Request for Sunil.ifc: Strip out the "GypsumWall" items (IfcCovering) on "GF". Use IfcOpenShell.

First a look at what the model holds.

```python
import ifcopenshell
import ifcopenshell.util.element

model = ifcopenshell.open("Sunil.ifc")
print(model.schema)
storey = next(s for s in model.by_type("IfcBuildingStorey") if s.Name == "GF")
coverings = [e for e in ifcopenshell.util.element.get_decomposition(storey) if e.is_a("IfcCovering")]
seen = {}
for e in coverings:
    element_type = ifcopenshell.util.element.get_type(e)
    name = element_type.Name if element_type not in (None, e) else None
    seen[name] = seen.get(name, 0) + 1
for name, count in sorted(seen.items(), key=str):
    print(count, "x", name)
```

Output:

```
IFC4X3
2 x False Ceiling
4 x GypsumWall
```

```python
import ifcopenshell
import ifcopenshell.api.root
import ifcopenshell.util.element

model = ifcopenshell.open("Sunil.ifc")

storey = next(s for s in model.by_type("IfcBuildingStorey") if s.Name == "GF")
coverings = [e for e in ifcopenshell.util.element.get_decomposition(storey) if e.is_a("IfcCovering")]
targets = [e for e in coverings if (t := ifcopenshell.util.element.get_type(e)) not in (None, e) and t.Name == "GypsumWall"]

for e in targets:
    ifcopenshell.api.root.remove_product(model, product=e)
print(len(targets), "removed")

model.write("Sunil_rev.ifc")
```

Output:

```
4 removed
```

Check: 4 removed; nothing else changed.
